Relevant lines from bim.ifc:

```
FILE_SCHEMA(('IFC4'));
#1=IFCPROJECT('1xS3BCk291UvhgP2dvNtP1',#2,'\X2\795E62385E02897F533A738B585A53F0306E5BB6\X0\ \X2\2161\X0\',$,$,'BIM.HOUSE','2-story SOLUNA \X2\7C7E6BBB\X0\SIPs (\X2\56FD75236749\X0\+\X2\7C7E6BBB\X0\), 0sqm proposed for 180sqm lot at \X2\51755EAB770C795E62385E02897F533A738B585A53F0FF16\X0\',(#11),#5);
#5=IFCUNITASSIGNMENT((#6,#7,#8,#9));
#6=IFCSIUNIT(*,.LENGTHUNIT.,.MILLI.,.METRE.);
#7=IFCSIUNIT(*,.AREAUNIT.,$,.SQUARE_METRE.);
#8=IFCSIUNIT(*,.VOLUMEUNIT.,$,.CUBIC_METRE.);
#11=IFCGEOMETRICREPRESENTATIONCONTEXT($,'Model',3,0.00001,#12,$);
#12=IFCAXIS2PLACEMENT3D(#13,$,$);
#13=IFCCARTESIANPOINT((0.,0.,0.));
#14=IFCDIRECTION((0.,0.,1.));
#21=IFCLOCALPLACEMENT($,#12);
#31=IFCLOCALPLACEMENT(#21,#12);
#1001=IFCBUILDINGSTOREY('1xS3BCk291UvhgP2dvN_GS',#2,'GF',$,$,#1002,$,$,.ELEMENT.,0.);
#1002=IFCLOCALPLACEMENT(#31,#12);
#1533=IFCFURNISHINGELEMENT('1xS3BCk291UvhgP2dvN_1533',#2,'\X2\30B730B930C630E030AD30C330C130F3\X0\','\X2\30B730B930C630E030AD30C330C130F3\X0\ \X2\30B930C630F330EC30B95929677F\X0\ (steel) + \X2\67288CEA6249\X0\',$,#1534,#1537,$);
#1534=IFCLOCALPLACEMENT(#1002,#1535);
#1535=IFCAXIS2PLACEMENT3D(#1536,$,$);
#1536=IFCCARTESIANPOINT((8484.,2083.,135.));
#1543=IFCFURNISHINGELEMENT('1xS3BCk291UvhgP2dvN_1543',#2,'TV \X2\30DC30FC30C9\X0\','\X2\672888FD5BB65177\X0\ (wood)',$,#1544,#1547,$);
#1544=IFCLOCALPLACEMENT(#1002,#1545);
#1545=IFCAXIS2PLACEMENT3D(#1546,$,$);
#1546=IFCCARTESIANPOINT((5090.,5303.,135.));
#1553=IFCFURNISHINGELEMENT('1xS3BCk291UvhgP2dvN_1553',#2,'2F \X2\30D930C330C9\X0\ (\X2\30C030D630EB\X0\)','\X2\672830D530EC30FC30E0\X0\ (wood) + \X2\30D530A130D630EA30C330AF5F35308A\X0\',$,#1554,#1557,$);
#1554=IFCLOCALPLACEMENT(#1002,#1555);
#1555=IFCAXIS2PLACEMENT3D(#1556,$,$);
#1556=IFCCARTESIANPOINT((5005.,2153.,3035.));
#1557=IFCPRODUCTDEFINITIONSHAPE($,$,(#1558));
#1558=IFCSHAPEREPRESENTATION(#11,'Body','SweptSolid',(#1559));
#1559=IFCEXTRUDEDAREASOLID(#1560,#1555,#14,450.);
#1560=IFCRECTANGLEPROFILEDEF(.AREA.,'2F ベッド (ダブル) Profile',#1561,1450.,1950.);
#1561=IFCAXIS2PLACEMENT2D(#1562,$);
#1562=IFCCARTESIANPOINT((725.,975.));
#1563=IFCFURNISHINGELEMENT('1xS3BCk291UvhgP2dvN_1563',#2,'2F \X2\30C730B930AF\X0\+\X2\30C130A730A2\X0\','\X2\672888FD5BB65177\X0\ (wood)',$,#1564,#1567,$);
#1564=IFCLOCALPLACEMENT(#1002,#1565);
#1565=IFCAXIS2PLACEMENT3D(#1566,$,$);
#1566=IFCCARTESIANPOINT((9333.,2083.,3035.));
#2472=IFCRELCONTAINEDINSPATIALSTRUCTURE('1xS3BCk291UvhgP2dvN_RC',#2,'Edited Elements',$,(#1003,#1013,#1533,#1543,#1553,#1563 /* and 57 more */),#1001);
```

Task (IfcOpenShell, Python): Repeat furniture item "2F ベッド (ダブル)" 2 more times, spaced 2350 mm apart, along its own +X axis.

```python
import ifcopenshell
import ifcopenshell.api.geometry
import ifcopenshell.api.root
import ifcopenshell.util.element
import ifcopenshell.util.placement
import ifcopenshell.util.unit

model = ifcopenshell.open("bim.ifc")
unit_scale = ifcopenshell.util.unit.calculate_unit_scale(model)


def reuse_history(source, copy):
    """copy_class also copies each property set's owner history, people and application; keep the originals."""
    for rel in copy.IsDefinedBy:
        if rel.is_a("IfcRelDefinesByProperties") and (history := rel.RelatingPropertyDefinition.OwnerHistory):
            rel.RelatingPropertyDefinition.OwnerHistory = source.OwnerHistory
            ifcopenshell.util.element.remove_deep2(model, history)


source = model.by_guid("1xS3BCk291UvhgP2dvN_1553")
base = ifcopenshell.util.placement.get_local_placement(source.ObjectPlacement)
step = base[:3, 0] * 2.35 / unit_scale

for i in range(1, 3):
    copy = ifcopenshell.api.root.copy_class(model, product=source)
    copy.Representation = ifcopenshell.util.element.copy_deep(
        model, source.Representation, exclude=["IfcGeometricRepresentationContext", "IfcRepresentationMap"]
    )
    reuse_history(source, copy)
    matrix = base.copy()
    matrix[:3, 3] += i * step
    print("added at", matrix[:3, 3].round(3) + 0.0)
    ifcopenshell.api.geometry.edit_object_placement(model, product=copy, matrix=matrix, is_si=False)

model.write("bim_updated.ifc")
```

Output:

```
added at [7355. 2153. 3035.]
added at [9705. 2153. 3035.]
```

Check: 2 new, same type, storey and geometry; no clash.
